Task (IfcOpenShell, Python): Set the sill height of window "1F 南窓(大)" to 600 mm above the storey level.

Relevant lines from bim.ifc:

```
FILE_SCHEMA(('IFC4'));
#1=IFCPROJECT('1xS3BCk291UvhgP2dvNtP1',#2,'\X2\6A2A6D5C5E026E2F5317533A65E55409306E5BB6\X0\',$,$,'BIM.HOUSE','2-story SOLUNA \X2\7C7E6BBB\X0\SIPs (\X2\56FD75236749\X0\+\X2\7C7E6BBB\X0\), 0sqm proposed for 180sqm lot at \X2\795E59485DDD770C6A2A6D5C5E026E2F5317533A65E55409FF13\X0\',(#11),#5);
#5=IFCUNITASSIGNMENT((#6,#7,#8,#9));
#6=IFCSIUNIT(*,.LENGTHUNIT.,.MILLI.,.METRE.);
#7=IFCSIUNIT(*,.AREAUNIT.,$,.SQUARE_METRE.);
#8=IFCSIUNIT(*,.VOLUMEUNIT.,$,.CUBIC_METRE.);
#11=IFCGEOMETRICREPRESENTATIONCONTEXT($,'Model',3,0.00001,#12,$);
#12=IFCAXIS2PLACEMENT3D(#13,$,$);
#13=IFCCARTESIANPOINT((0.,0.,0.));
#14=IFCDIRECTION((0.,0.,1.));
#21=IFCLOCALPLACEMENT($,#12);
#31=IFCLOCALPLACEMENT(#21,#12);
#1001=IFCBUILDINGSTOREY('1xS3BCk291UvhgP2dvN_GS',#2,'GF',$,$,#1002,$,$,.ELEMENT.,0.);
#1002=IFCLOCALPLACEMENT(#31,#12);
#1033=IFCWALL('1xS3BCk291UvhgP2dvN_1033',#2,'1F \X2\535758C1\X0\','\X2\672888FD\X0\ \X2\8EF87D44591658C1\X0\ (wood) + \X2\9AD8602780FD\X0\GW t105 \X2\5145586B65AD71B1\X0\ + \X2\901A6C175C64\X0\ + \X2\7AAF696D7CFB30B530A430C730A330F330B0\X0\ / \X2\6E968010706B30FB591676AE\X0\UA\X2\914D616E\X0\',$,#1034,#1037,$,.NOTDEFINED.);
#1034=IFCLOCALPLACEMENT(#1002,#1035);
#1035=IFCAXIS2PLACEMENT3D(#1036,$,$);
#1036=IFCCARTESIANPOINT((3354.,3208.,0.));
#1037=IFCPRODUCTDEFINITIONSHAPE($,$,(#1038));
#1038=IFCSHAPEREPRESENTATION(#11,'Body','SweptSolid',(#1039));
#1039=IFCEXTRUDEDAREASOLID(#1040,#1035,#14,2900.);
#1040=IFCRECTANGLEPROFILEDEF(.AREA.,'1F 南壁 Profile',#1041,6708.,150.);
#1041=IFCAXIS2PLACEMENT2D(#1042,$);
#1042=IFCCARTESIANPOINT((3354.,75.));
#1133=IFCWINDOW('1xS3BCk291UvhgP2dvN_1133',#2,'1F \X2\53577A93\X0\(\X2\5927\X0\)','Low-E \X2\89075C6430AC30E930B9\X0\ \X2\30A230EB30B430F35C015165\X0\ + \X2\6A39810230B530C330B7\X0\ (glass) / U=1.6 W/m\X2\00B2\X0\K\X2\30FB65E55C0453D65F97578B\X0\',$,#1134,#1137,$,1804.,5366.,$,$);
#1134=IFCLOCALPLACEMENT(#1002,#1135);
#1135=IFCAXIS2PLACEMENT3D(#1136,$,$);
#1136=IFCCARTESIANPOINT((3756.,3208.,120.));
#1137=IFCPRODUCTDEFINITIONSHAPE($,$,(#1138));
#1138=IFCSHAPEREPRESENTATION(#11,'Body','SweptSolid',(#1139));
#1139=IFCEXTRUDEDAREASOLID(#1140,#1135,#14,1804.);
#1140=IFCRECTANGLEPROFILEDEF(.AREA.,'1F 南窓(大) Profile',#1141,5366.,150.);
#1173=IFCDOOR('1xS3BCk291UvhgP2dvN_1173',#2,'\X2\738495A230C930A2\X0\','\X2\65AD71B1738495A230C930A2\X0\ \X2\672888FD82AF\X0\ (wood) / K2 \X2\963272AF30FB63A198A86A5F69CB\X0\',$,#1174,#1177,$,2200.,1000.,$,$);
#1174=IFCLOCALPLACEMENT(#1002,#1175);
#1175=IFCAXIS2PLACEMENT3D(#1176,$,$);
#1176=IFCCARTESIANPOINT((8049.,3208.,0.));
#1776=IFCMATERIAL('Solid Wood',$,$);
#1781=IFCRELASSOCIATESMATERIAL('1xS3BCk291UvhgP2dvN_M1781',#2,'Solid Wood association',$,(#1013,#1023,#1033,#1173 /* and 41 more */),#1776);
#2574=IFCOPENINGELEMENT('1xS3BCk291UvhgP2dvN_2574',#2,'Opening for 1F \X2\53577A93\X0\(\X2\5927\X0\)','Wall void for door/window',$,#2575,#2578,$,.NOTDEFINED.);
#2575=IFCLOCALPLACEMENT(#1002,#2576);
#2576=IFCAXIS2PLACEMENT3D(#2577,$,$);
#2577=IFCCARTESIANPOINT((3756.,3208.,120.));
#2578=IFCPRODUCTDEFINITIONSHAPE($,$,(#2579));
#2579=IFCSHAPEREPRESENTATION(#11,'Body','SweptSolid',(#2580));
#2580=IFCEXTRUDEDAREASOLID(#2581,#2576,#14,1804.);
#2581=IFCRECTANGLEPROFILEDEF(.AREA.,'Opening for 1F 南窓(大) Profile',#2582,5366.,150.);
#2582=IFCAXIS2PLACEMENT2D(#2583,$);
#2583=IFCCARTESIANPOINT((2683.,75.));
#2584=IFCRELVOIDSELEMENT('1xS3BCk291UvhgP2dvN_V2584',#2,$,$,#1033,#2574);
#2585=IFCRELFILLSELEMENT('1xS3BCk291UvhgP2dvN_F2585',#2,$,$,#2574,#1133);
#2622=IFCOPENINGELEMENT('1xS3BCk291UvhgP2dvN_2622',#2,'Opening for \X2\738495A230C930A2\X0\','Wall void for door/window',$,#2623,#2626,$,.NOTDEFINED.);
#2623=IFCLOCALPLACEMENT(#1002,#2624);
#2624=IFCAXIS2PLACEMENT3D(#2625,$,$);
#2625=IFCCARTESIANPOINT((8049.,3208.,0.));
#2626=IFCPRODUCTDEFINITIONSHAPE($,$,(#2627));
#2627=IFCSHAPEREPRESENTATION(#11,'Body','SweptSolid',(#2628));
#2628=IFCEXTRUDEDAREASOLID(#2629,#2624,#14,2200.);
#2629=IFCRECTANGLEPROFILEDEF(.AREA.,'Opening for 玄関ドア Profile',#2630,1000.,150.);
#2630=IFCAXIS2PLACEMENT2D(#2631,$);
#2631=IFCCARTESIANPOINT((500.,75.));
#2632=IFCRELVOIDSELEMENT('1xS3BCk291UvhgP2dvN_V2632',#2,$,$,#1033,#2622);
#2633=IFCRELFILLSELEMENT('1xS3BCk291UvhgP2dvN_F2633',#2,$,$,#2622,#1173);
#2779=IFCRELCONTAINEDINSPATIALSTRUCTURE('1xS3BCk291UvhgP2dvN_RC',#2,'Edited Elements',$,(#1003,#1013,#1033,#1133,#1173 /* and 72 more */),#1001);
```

```python
import numpy as np
import ifcopenshell
import ifcopenshell.api.geometry
import ifcopenshell.geom
import ifcopenshell.util.element
import ifcopenshell.util.placement
import ifcopenshell.util.shape
import ifcopenshell.util.unit

model = ifcopenshell.open("bim.ifc")
unit_scale = ifcopenshell.util.unit.calculate_unit_scale(model)

window = model.by_guid("1xS3BCk291UvhgP2dvN_1133")
opening = window.FillsVoids[0].RelatingOpeningElement
storey = ifcopenshell.util.element.get_container(window, ifc_class="IfcBuildingStorey")
level = ifcopenshell.util.placement.get_local_placement(storey.ObjectPlacement)[2, 3]

# The opening's origin need not be at the sill, so measure its lowest point.
shape = ifcopenshell.geom.create_shape(ifcopenshell.geom.settings(), opening)
bottom = ifcopenshell.util.shape.get_shape_bottom_elevation(shape, shape.geometry) / unit_scale
dz = level + 0.6 / unit_scale - bottom

shift = np.array([0.0, 0.0, dz])
# The window is not placed relative to its opening, so move both.
for product in (opening, window):
    matrix = ifcopenshell.util.placement.get_local_placement(product.ObjectPlacement)
    matrix[:3, 3] += shift
    ifcopenshell.api.geometry.edit_object_placement(model, product=product, matrix=matrix, is_si=False)

print(f"moved by {dz * unit_scale:+.3f} m")

model.write("bim_rev.ifc")
```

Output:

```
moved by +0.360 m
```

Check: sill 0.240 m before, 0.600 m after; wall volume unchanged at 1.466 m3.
